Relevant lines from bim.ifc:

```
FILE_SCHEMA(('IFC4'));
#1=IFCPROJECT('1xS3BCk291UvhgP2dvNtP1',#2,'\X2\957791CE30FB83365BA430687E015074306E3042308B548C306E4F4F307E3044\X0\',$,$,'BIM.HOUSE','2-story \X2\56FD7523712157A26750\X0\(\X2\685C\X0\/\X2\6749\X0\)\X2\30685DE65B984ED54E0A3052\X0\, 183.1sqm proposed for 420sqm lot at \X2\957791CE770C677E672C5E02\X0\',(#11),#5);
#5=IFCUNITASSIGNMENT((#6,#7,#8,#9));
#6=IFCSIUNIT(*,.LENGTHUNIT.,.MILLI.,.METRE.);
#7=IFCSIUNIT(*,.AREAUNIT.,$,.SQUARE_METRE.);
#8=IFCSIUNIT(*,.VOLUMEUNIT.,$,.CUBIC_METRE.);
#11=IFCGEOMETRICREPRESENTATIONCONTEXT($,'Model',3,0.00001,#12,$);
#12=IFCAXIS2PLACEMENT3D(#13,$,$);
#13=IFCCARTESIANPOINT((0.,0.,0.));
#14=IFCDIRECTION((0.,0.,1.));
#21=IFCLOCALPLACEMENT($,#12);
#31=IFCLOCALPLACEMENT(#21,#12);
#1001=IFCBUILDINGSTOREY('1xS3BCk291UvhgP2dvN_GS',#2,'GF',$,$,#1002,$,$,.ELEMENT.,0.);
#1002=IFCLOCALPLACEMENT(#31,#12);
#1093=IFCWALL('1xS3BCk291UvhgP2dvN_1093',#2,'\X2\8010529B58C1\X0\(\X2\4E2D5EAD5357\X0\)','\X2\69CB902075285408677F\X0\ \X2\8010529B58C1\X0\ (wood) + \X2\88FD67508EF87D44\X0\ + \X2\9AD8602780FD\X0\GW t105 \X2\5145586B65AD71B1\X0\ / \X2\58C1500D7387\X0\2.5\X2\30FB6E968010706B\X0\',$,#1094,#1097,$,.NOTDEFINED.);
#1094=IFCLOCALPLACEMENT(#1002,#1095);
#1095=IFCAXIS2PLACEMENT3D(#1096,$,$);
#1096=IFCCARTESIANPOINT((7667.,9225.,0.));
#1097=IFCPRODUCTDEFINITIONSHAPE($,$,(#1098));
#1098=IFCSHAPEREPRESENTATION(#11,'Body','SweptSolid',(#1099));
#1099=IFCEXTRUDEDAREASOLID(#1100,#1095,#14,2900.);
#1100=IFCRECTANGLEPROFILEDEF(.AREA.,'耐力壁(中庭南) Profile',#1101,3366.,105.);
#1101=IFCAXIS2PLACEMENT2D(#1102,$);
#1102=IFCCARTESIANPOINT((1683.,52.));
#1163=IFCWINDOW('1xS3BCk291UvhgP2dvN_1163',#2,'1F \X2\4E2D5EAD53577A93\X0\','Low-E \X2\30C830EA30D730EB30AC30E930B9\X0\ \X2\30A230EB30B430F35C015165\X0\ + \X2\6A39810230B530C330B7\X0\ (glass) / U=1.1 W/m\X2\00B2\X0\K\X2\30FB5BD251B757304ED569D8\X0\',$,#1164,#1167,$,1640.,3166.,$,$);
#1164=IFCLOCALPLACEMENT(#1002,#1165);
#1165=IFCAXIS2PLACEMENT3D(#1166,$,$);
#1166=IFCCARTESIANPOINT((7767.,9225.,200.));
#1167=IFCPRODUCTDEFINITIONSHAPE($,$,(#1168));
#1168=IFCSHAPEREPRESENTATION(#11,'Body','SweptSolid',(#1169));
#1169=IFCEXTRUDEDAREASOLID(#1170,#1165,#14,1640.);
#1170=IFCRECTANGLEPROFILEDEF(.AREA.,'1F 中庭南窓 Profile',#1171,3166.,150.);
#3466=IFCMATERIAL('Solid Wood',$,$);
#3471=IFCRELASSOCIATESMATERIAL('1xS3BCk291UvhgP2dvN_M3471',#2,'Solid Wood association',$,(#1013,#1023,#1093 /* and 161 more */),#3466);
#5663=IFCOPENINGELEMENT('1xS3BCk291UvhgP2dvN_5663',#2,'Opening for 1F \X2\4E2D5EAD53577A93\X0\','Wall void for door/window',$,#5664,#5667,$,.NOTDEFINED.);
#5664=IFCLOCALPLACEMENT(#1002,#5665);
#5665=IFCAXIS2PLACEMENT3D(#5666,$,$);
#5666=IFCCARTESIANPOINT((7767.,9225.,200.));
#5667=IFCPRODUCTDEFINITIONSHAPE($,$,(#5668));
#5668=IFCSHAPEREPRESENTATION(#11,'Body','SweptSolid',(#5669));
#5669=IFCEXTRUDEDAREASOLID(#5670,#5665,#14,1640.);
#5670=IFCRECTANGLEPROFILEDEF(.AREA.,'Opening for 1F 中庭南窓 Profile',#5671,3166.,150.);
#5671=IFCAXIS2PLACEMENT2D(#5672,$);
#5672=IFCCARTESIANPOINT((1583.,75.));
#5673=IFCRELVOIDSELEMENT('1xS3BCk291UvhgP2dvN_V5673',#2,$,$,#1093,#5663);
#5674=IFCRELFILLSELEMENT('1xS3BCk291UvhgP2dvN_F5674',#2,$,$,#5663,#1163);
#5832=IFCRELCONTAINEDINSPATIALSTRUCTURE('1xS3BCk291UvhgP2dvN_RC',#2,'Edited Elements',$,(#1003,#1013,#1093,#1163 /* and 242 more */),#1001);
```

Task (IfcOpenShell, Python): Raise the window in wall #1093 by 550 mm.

```python
import numpy as np
import ifcopenshell
import ifcopenshell.api.geometry
import ifcopenshell.util.placement
import ifcopenshell.util.unit

model = ifcopenshell.open("bim.ifc")
unit_scale = ifcopenshell.util.unit.calculate_unit_scale(model)

window = model.by_guid("1xS3BCk291UvhgP2dvN_1163")
opening = window.FillsVoids[0].RelatingOpeningElement
dz = 0.55 / unit_scale

shift = np.array([0.0, 0.0, dz])
# The window is not placed relative to its opening, so move both.
for product in (opening, window):
    matrix = ifcopenshell.util.placement.get_local_placement(product.ObjectPlacement)
    matrix[:3, 3] += shift
    ifcopenshell.api.geometry.edit_object_placement(model, product=product, matrix=matrix, is_si=False)

print(f"moved by {dz * unit_scale:+.3f} m")

model.write("bim_edited.ifc")
```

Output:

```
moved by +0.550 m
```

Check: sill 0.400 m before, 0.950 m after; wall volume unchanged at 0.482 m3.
